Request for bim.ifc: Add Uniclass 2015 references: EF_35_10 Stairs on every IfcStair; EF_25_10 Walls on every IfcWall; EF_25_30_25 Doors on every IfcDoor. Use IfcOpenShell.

First a look at what the model holds.

```python
import ifcopenshell

model = ifcopenshell.open("bim.ifc")
print(model.schema)
print("classifications:", [c.Name for c in model.by_type("IfcClassification")])
for ifc_class in ("IfcDoor", "IfcRoof", "IfcStair", "IfcWall", "IfcWindow"):
    print(ifc_class, len(model.by_type(ifc_class)))
```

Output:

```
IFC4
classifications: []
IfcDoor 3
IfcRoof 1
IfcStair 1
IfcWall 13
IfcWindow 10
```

```python
import ifcopenshell
import ifcopenshell.api.classification

model = ifcopenshell.open("bim.ifc")

system = ifcopenshell.api.classification.add_classification(model, classification="Uniclass 2015")

codes = {
    "IfcStair": ("EF_35_10", "Stairs"),
    "IfcWall": ("EF_25_10", "Walls"),
    "IfcDoor": ("EF_25_30_25", "Doors"),
}
for ifc_class, (code, name) in codes.items():
    products = model.by_type(ifc_class)
    ifcopenshell.api.classification.add_reference(
        model, products=products, classification=system, identification=code, name=name
    )
    print(code, len(products))

model.write("bim-out.ifc")
```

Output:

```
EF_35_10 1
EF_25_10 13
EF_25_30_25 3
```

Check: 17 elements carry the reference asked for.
